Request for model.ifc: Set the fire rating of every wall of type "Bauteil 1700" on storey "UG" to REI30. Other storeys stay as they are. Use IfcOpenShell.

First a look at what the model holds.

```python
import ifcopenshell
import ifcopenshell.util.element

model = ifcopenshell.open("model.ifc")
print(model.schema)
storey = next(s for s in model.by_type("IfcBuildingStorey") if s.Name == "UG")
walls = [e for e in ifcopenshell.util.element.get_decomposition(storey) if e.is_a("IfcWall")]
seen = {}
for e in walls:
    element_type = ifcopenshell.util.element.get_type(e)
    key = (element_type.Name if element_type != e and element_type else None, ifcopenshell.util.element.get_pset(e, "Pset_WallCommon", "FireRating"))
    seen[key] = seen.get(key, 0) + 1
for (name, value), count in sorted(seen.items(), key=str):
    print(count, "x", name, "|", value)
```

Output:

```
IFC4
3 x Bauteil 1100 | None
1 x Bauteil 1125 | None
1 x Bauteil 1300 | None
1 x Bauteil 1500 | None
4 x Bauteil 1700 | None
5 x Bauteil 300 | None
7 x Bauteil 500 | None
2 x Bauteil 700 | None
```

```python
import ifcopenshell
import ifcopenshell.api.pset
import ifcopenshell.util.element

model = ifcopenshell.open("model.ifc")

storey = next(s for s in model.by_type("IfcBuildingStorey") if s.Name == "UG")
walls = [e for e in ifcopenshell.util.element.get_decomposition(storey) if e.is_a("IfcWall")]

count = 0
for e in walls:
    element_type = ifcopenshell.util.element.get_type(e)
    if element_type in (None, e) or element_type.Name != "Bauteil 1700":
        continue
    # add_pset returns the element's existing set when there is one.
    pset = ifcopenshell.api.pset.add_pset(model, product=e, name="Pset_WallCommon")
    ifcopenshell.api.pset.edit_pset(model, pset=pset, properties={"FireRating": "REI30"})
    count += 1

print(count, "walls updated")

model.write("model_edited.ifc")
```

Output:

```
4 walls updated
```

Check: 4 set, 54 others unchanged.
